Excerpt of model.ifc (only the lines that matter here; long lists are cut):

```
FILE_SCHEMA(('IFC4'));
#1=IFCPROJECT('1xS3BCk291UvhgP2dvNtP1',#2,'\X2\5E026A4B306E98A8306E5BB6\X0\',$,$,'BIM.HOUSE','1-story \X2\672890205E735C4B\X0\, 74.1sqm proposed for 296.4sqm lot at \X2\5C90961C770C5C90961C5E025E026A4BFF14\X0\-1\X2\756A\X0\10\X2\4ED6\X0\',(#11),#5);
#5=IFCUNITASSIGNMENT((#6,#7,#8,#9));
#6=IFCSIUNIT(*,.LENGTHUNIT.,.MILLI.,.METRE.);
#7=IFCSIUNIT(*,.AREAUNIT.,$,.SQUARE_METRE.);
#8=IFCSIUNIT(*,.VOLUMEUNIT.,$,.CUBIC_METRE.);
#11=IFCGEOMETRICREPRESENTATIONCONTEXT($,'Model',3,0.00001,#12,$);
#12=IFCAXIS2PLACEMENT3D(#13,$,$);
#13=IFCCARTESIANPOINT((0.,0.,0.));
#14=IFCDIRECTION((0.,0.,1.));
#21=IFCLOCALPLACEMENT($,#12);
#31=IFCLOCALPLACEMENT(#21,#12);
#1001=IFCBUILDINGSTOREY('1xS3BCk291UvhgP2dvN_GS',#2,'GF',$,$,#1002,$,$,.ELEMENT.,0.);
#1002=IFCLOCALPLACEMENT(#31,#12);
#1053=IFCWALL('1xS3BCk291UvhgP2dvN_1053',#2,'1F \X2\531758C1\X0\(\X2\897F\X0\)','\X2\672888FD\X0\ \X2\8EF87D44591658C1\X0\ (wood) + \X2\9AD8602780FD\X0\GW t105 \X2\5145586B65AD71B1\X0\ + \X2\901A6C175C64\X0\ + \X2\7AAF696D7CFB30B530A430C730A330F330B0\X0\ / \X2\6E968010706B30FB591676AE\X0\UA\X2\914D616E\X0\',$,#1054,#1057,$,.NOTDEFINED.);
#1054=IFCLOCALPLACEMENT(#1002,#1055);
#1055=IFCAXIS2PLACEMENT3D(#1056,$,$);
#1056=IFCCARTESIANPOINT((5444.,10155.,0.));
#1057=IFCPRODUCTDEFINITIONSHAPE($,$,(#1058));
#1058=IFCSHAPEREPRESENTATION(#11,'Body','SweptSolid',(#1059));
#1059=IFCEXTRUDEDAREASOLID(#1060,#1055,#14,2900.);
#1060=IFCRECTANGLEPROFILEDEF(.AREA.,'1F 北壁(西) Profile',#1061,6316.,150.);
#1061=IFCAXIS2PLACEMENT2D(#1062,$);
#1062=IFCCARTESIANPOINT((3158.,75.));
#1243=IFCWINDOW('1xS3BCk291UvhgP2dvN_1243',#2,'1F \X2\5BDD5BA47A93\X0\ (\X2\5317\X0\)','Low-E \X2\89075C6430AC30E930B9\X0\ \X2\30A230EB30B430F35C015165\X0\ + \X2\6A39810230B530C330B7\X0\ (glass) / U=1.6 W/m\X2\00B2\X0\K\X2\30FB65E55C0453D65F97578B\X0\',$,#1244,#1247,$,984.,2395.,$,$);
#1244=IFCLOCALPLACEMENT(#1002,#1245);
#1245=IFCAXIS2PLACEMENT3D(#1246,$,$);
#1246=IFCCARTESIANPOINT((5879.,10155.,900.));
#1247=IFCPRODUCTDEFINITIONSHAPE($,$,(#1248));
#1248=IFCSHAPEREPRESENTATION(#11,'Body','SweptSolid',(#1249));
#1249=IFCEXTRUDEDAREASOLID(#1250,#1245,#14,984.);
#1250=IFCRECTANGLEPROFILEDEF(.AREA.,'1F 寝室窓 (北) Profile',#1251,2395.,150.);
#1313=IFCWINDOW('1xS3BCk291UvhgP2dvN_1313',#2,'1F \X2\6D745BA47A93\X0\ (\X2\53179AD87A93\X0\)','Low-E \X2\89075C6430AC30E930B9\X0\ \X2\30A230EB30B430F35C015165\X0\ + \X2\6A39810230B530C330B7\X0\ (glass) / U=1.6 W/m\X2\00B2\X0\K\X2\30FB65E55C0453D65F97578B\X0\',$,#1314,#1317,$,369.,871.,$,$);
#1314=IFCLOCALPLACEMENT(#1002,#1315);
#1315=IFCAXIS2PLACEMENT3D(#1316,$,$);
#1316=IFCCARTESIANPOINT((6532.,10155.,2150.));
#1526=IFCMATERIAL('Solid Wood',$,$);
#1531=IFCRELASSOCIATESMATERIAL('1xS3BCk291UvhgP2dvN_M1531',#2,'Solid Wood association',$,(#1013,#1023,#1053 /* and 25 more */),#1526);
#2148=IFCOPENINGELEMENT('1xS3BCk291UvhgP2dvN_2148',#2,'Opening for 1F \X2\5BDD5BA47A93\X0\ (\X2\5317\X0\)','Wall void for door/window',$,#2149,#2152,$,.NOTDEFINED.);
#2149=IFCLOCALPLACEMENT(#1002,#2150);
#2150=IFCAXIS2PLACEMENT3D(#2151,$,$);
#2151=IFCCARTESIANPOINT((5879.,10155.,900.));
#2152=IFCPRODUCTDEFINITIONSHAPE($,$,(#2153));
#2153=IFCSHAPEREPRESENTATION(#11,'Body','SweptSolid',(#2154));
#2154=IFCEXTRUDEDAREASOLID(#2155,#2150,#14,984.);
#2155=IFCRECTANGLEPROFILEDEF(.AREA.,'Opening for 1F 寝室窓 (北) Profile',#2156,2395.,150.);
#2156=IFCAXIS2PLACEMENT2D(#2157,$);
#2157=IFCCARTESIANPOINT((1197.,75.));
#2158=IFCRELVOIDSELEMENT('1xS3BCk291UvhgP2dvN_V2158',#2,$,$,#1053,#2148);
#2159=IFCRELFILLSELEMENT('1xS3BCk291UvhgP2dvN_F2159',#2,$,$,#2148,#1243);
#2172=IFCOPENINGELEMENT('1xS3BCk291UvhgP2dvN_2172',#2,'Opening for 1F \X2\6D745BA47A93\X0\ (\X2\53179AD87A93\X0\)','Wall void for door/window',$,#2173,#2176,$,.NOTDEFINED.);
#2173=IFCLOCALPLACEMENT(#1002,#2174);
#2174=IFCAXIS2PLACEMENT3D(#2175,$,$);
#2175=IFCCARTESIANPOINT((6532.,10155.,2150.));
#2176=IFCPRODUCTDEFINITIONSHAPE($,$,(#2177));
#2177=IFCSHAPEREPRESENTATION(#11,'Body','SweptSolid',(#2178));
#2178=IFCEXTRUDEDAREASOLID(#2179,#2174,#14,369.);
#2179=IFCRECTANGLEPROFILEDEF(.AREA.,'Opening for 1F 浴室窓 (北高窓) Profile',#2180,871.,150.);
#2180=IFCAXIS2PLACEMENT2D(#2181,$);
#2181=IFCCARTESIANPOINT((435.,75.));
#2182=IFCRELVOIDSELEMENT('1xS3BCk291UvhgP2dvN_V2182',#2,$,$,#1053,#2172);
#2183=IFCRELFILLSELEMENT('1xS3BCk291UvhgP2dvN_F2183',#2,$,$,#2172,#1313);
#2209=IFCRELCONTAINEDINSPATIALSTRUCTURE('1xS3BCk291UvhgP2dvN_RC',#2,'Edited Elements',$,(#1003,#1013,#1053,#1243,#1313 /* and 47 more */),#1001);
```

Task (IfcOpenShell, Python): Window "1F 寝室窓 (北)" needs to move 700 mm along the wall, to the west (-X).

```python
import ifcopenshell
import ifcopenshell.api.geometry
import ifcopenshell.util.placement

model = ifcopenshell.open("model.ifc")

window = model.by_id(1243)
opening = window.FillsVoids[0].RelatingOpeningElement
wall = opening.VoidsElements[0].RelatingBuildingElement

wall_matrix = ifcopenshell.util.placement.get_local_placement(wall.ObjectPlacement)
shift = wall_matrix[:3, 0] * -700.0
before = ifcopenshell.util.placement.get_local_placement(window.ObjectPlacement)[:3, 3].copy()

# The window is not placed relative to its opening, so move both.
for product in (opening, window):
    matrix = ifcopenshell.util.placement.get_local_placement(product.ObjectPlacement)
    matrix[:3, 3] += shift
    ifcopenshell.api.geometry.edit_object_placement(model, product=product, matrix=matrix, is_si=False)

after = ifcopenshell.util.placement.get_local_placement(window.ObjectPlacement)[:3, 3]
print("window moved by", (after - before).round(3) + 0.0)

model.write("model_rev.ifc")
```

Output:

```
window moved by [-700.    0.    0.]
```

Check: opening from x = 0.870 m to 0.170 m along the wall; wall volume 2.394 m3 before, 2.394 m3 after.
